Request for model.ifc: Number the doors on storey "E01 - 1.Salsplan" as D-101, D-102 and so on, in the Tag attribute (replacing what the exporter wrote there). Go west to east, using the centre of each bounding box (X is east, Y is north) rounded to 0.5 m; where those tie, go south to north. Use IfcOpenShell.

First a look at what the model holds.

```python
import ifcopenshell
import ifcopenshell.util.element
import ifcopenshell.util.placement

model = ifcopenshell.open("model.ifc")
print(model.schema)
storey = next(s for s in model.by_type("IfcBuildingStorey") if s.Name == "E01 - 1.Salsplan")
doors = [e for e in ifcopenshell.util.element.get_decomposition(storey) if e.is_a("IfcDoor")]
for e in sorted(doors, key=lambda e: e.id()):
    origin = ifcopenshell.util.placement.get_local_placement(e.ObjectPlacement)[:3, 3]
    print(e.id(), e.Tag, e.Name, origin.round(2) + 0.0, sep=" | ")
```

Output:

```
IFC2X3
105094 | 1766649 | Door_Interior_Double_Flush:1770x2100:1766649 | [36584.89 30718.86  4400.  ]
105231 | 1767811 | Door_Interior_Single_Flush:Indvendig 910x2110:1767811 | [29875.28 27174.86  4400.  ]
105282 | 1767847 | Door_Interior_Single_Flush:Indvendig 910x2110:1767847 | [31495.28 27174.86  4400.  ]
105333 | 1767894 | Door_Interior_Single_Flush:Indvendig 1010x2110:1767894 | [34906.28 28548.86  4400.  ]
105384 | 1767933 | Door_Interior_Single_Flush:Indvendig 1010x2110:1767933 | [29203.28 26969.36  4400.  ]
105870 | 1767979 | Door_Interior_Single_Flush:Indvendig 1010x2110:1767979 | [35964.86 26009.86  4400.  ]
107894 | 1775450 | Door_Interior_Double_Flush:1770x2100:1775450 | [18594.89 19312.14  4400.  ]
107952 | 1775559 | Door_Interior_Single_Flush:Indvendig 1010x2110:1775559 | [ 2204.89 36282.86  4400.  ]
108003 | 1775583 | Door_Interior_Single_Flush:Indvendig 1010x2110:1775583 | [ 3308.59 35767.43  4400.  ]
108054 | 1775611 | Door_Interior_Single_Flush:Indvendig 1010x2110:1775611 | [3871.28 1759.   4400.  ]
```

```python
import ifcopenshell
import ifcopenshell.geom
import ifcopenshell.util.element
import ifcopenshell.util.shape

model = ifcopenshell.open("model.ifc")
settings = ifcopenshell.geom.settings()
settings.set("use-world-coords", True)


def centre(element):
    shape = ifcopenshell.geom.create_shape(settings, element)
    return ifcopenshell.util.shape.get_bbox_centroid(shape.geometry)


storey = next(s for s in model.by_type("IfcBuildingStorey") if s.Name == "E01 - 1.Salsplan")
doors = [e for e in ifcopenshell.util.element.get_decomposition(storey) if e.is_a("IfcDoor")]

# Insertion points can sit at a corner or the storey origin, so sort by the geometry (in metres).
centres = {e: centre(e) for e in doors}
doors.sort(key=lambda e: (round(centres[e][0] / 0.5), centres[e][1]))

for i, e in enumerate(doors, start=1):
    number = f"D-1{i:02d}"
    e.Tag = number
    print(e.id(), number)

model.write("model_v2.ifc")
```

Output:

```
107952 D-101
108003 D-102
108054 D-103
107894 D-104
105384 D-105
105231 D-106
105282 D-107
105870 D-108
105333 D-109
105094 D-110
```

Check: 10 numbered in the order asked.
